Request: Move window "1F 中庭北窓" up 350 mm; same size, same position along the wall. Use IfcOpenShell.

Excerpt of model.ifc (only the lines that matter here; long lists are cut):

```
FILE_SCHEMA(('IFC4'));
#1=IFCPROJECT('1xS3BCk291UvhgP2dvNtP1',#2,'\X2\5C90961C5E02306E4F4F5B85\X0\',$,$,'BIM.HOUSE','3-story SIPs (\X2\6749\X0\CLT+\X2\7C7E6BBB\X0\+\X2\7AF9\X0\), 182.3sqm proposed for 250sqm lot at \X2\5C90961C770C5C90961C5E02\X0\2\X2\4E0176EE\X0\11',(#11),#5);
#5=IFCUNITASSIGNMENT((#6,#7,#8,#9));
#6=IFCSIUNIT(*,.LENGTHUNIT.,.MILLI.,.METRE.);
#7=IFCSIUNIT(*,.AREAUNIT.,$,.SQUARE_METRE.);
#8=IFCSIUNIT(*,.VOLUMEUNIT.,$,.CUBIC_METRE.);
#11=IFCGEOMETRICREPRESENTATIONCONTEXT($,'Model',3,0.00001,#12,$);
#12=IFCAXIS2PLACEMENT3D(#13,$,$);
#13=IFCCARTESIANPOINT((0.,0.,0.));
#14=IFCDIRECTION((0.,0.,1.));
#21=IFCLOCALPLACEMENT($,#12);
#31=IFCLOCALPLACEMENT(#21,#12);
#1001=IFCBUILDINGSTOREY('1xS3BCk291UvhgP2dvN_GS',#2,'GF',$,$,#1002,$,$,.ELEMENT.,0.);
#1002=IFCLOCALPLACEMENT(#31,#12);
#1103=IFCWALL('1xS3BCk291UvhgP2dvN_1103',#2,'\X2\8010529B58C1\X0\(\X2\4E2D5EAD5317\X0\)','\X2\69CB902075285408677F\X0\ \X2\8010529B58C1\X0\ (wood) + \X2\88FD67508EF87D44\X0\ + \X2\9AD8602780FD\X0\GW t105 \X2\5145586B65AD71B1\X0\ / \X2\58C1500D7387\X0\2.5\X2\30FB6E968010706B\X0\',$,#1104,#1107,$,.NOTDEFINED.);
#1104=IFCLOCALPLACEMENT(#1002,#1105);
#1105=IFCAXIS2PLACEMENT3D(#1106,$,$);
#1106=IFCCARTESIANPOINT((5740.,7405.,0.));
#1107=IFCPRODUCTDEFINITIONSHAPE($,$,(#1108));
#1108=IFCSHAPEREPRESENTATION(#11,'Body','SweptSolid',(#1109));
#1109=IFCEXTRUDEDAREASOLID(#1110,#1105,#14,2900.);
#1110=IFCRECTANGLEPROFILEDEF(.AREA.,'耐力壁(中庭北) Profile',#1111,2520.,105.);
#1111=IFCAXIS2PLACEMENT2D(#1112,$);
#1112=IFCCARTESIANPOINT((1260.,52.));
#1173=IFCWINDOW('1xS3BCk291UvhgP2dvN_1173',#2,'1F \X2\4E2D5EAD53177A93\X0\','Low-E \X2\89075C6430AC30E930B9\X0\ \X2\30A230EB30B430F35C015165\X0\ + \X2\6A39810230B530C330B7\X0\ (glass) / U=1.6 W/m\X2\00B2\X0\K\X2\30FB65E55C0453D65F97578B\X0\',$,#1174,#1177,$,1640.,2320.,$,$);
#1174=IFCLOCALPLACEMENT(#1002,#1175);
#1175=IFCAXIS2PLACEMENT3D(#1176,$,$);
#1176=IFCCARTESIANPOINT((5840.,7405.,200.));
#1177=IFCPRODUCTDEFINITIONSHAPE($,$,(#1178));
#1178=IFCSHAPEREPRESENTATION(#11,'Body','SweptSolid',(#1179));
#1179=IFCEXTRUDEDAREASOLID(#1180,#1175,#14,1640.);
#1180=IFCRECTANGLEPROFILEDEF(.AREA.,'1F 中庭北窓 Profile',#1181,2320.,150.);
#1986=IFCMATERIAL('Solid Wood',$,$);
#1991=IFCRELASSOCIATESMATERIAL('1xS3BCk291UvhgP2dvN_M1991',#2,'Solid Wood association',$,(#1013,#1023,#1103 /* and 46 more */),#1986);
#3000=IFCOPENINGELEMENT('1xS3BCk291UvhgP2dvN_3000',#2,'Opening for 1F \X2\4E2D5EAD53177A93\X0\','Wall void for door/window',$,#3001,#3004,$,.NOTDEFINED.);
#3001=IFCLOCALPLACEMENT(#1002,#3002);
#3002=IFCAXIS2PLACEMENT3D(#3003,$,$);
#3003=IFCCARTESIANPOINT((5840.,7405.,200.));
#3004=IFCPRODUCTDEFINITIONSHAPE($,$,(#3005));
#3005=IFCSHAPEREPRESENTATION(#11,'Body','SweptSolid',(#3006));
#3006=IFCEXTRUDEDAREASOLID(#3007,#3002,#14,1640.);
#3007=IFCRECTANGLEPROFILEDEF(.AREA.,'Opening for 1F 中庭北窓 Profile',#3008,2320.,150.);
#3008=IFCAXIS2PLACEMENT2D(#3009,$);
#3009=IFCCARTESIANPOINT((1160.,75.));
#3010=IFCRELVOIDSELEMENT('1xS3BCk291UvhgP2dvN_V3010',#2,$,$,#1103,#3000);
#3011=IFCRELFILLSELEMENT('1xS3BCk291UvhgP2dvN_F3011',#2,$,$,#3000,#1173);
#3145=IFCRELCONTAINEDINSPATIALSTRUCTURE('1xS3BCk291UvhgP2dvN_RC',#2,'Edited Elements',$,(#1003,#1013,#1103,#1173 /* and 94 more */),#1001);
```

```python
import numpy as np
import ifcopenshell
import ifcopenshell.api.geometry
import ifcopenshell.util.placement
import ifcopenshell.util.unit

model = ifcopenshell.open("model.ifc")
unit_scale = ifcopenshell.util.unit.calculate_unit_scale(model)

window = model.by_guid("1xS3BCk291UvhgP2dvN_1173")
opening = window.FillsVoids[0].RelatingOpeningElement
dz = 0.35 / unit_scale

shift = np.array([0.0, 0.0, dz])
# The window is not placed relative to its opening, so move both.
for product in (opening, window):
    matrix = ifcopenshell.util.placement.get_local_placement(product.ObjectPlacement)
    matrix[:3, 3] += shift
    ifcopenshell.api.geometry.edit_object_placement(model, product=product, matrix=matrix, is_si=False)

print(f"moved by {dz * unit_scale:+.3f} m")

model.write("model_updated.ifc")
```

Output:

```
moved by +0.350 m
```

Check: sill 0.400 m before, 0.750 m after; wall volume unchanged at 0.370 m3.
